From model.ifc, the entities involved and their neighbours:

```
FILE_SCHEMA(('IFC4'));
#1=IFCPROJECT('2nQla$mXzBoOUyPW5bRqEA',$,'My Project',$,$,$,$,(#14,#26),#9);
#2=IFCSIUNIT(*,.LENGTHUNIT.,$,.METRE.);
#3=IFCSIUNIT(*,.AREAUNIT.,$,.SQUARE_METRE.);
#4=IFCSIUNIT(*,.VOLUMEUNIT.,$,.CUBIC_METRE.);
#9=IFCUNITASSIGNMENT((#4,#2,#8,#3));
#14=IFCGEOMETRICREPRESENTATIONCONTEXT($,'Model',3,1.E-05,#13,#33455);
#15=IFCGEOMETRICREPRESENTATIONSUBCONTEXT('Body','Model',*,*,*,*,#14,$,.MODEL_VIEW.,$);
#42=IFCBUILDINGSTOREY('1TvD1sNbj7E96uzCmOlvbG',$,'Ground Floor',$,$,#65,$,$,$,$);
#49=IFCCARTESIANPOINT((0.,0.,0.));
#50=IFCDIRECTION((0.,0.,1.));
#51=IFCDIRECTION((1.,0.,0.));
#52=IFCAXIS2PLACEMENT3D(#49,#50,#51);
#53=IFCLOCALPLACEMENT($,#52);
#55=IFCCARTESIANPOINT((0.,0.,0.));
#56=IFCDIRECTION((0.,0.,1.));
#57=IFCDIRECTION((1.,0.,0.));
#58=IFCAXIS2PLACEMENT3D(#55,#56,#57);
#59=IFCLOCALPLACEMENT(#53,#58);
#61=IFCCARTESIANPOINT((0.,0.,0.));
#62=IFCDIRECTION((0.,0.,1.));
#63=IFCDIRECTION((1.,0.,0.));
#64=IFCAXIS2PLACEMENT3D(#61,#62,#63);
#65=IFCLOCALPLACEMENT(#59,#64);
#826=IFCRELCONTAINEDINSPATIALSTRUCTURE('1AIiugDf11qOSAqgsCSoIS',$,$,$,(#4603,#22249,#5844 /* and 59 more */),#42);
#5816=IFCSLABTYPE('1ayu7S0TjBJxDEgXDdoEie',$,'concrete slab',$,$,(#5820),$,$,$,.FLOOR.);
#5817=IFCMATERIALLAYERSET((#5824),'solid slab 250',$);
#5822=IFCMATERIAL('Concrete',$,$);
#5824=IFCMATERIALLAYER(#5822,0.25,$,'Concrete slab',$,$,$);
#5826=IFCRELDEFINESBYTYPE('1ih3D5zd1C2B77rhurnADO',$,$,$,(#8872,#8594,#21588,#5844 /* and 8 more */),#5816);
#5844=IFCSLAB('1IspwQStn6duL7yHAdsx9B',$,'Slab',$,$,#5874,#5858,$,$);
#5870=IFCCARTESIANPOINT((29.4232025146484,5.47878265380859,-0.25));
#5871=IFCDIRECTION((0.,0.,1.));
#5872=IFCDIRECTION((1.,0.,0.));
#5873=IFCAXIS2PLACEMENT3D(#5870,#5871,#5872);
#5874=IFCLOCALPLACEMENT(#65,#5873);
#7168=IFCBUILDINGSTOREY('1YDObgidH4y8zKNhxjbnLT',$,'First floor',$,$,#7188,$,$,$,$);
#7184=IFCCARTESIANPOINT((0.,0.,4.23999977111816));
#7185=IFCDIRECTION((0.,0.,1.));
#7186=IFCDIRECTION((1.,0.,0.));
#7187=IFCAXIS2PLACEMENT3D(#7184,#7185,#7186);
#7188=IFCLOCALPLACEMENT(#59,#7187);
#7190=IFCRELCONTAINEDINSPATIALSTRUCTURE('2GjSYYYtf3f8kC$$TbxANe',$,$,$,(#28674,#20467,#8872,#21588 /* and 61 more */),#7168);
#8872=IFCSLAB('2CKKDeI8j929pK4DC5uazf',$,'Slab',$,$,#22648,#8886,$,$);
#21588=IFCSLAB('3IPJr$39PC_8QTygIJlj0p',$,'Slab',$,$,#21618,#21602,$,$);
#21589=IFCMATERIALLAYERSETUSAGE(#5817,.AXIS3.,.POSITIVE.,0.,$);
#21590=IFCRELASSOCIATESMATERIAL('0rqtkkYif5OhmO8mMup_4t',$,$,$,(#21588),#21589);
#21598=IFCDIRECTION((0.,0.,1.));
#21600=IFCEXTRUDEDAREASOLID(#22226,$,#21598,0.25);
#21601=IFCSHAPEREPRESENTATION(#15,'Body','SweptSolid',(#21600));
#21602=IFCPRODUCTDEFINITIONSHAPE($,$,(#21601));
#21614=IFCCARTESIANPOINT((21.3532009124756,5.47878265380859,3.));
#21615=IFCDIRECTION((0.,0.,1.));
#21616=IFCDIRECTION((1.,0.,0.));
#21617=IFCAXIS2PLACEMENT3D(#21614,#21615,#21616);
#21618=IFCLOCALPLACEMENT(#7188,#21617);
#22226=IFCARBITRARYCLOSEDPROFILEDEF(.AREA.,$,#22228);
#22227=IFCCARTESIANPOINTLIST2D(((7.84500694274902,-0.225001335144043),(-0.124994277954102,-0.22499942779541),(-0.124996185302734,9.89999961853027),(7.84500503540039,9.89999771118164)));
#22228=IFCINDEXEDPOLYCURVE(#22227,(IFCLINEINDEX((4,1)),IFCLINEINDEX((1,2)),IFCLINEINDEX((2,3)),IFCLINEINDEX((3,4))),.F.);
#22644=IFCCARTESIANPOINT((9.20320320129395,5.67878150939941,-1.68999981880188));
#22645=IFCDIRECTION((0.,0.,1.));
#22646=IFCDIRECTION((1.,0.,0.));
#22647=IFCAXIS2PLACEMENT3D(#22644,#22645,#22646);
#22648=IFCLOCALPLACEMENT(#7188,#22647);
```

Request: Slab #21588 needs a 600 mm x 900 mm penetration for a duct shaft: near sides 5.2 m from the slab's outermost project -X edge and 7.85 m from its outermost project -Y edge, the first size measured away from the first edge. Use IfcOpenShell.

```python
import numpy as np
import ifcopenshell
import ifcopenshell.api.feature
import ifcopenshell.api.geometry
import ifcopenshell.api.root
import ifcopenshell.geom
import ifcopenshell.util.placement
import ifcopenshell.util.representation
import ifcopenshell.util.shape
import ifcopenshell.util.unit

model = ifcopenshell.open("model.ifc")
unit_scale = ifcopenshell.util.unit.calculate_unit_scale(model)
settings = ifcopenshell.geom.settings()


def volume(element):
    """Net volume in cubic metres, openings subtracted."""
    shape = ifcopenshell.geom.create_shape(settings, element)
    return ifcopenshell.util.shape.get_volume(shape.geometry)


slab = model.by_guid("3IPJr$39PC_8QTygIJlj0p")
before = volume(slab)

# Extent in the slab's own axes, in metres. The edges named are its -X and -Y sides.
slab_shape = ifcopenshell.geom.create_shape(settings, slab)
vertices = ifcopenshell.util.shape.get_vertices(slab_shape.geometry)
x_min, y_min, bottom = vertices.min(axis=0)
top = vertices[:, 2].max()

opening = ifcopenshell.api.root.create_entity(model, ifc_class="IfcOpeningElement", name="Duct shaft opening", predefined_type="OPENING")
context = ifcopenshell.util.representation.get_context(model, "Model", "Body", "MODEL_VIEW")
width, depth = 0.6, 0.9
outline = [(0.0, 0.0), (width, 0.0), (width, depth), (0.0, depth), (0.0, 0.0)]
# Overshoot both faces by 50 mm so the cut is clean.
shape = ifcopenshell.api.geometry.add_slab_representation(
    model, context=context, depth=top - bottom + 0.1, polyline=outline
)
ifcopenshell.api.geometry.assign_representation(model, product=opening, representation=shape)

matrix = ifcopenshell.util.placement.get_local_placement(slab.ObjectPlacement)
matrix[:, 3] = matrix @ np.append(np.array([x_min + 5.2, y_min + 7.85, bottom - 0.05]) / unit_scale, 1.0)
ifcopenshell.api.geometry.edit_object_placement(model, product=opening, matrix=matrix, is_si=False)
ifcopenshell.api.feature.add_feature(model, feature=opening, element=slab)

after = volume(slab)

print(f"slab volume {before:.3f} -> {after:.3f} m3")

model.write("model_updated.ifc")
```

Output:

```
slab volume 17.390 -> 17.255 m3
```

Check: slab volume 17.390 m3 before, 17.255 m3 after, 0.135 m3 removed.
